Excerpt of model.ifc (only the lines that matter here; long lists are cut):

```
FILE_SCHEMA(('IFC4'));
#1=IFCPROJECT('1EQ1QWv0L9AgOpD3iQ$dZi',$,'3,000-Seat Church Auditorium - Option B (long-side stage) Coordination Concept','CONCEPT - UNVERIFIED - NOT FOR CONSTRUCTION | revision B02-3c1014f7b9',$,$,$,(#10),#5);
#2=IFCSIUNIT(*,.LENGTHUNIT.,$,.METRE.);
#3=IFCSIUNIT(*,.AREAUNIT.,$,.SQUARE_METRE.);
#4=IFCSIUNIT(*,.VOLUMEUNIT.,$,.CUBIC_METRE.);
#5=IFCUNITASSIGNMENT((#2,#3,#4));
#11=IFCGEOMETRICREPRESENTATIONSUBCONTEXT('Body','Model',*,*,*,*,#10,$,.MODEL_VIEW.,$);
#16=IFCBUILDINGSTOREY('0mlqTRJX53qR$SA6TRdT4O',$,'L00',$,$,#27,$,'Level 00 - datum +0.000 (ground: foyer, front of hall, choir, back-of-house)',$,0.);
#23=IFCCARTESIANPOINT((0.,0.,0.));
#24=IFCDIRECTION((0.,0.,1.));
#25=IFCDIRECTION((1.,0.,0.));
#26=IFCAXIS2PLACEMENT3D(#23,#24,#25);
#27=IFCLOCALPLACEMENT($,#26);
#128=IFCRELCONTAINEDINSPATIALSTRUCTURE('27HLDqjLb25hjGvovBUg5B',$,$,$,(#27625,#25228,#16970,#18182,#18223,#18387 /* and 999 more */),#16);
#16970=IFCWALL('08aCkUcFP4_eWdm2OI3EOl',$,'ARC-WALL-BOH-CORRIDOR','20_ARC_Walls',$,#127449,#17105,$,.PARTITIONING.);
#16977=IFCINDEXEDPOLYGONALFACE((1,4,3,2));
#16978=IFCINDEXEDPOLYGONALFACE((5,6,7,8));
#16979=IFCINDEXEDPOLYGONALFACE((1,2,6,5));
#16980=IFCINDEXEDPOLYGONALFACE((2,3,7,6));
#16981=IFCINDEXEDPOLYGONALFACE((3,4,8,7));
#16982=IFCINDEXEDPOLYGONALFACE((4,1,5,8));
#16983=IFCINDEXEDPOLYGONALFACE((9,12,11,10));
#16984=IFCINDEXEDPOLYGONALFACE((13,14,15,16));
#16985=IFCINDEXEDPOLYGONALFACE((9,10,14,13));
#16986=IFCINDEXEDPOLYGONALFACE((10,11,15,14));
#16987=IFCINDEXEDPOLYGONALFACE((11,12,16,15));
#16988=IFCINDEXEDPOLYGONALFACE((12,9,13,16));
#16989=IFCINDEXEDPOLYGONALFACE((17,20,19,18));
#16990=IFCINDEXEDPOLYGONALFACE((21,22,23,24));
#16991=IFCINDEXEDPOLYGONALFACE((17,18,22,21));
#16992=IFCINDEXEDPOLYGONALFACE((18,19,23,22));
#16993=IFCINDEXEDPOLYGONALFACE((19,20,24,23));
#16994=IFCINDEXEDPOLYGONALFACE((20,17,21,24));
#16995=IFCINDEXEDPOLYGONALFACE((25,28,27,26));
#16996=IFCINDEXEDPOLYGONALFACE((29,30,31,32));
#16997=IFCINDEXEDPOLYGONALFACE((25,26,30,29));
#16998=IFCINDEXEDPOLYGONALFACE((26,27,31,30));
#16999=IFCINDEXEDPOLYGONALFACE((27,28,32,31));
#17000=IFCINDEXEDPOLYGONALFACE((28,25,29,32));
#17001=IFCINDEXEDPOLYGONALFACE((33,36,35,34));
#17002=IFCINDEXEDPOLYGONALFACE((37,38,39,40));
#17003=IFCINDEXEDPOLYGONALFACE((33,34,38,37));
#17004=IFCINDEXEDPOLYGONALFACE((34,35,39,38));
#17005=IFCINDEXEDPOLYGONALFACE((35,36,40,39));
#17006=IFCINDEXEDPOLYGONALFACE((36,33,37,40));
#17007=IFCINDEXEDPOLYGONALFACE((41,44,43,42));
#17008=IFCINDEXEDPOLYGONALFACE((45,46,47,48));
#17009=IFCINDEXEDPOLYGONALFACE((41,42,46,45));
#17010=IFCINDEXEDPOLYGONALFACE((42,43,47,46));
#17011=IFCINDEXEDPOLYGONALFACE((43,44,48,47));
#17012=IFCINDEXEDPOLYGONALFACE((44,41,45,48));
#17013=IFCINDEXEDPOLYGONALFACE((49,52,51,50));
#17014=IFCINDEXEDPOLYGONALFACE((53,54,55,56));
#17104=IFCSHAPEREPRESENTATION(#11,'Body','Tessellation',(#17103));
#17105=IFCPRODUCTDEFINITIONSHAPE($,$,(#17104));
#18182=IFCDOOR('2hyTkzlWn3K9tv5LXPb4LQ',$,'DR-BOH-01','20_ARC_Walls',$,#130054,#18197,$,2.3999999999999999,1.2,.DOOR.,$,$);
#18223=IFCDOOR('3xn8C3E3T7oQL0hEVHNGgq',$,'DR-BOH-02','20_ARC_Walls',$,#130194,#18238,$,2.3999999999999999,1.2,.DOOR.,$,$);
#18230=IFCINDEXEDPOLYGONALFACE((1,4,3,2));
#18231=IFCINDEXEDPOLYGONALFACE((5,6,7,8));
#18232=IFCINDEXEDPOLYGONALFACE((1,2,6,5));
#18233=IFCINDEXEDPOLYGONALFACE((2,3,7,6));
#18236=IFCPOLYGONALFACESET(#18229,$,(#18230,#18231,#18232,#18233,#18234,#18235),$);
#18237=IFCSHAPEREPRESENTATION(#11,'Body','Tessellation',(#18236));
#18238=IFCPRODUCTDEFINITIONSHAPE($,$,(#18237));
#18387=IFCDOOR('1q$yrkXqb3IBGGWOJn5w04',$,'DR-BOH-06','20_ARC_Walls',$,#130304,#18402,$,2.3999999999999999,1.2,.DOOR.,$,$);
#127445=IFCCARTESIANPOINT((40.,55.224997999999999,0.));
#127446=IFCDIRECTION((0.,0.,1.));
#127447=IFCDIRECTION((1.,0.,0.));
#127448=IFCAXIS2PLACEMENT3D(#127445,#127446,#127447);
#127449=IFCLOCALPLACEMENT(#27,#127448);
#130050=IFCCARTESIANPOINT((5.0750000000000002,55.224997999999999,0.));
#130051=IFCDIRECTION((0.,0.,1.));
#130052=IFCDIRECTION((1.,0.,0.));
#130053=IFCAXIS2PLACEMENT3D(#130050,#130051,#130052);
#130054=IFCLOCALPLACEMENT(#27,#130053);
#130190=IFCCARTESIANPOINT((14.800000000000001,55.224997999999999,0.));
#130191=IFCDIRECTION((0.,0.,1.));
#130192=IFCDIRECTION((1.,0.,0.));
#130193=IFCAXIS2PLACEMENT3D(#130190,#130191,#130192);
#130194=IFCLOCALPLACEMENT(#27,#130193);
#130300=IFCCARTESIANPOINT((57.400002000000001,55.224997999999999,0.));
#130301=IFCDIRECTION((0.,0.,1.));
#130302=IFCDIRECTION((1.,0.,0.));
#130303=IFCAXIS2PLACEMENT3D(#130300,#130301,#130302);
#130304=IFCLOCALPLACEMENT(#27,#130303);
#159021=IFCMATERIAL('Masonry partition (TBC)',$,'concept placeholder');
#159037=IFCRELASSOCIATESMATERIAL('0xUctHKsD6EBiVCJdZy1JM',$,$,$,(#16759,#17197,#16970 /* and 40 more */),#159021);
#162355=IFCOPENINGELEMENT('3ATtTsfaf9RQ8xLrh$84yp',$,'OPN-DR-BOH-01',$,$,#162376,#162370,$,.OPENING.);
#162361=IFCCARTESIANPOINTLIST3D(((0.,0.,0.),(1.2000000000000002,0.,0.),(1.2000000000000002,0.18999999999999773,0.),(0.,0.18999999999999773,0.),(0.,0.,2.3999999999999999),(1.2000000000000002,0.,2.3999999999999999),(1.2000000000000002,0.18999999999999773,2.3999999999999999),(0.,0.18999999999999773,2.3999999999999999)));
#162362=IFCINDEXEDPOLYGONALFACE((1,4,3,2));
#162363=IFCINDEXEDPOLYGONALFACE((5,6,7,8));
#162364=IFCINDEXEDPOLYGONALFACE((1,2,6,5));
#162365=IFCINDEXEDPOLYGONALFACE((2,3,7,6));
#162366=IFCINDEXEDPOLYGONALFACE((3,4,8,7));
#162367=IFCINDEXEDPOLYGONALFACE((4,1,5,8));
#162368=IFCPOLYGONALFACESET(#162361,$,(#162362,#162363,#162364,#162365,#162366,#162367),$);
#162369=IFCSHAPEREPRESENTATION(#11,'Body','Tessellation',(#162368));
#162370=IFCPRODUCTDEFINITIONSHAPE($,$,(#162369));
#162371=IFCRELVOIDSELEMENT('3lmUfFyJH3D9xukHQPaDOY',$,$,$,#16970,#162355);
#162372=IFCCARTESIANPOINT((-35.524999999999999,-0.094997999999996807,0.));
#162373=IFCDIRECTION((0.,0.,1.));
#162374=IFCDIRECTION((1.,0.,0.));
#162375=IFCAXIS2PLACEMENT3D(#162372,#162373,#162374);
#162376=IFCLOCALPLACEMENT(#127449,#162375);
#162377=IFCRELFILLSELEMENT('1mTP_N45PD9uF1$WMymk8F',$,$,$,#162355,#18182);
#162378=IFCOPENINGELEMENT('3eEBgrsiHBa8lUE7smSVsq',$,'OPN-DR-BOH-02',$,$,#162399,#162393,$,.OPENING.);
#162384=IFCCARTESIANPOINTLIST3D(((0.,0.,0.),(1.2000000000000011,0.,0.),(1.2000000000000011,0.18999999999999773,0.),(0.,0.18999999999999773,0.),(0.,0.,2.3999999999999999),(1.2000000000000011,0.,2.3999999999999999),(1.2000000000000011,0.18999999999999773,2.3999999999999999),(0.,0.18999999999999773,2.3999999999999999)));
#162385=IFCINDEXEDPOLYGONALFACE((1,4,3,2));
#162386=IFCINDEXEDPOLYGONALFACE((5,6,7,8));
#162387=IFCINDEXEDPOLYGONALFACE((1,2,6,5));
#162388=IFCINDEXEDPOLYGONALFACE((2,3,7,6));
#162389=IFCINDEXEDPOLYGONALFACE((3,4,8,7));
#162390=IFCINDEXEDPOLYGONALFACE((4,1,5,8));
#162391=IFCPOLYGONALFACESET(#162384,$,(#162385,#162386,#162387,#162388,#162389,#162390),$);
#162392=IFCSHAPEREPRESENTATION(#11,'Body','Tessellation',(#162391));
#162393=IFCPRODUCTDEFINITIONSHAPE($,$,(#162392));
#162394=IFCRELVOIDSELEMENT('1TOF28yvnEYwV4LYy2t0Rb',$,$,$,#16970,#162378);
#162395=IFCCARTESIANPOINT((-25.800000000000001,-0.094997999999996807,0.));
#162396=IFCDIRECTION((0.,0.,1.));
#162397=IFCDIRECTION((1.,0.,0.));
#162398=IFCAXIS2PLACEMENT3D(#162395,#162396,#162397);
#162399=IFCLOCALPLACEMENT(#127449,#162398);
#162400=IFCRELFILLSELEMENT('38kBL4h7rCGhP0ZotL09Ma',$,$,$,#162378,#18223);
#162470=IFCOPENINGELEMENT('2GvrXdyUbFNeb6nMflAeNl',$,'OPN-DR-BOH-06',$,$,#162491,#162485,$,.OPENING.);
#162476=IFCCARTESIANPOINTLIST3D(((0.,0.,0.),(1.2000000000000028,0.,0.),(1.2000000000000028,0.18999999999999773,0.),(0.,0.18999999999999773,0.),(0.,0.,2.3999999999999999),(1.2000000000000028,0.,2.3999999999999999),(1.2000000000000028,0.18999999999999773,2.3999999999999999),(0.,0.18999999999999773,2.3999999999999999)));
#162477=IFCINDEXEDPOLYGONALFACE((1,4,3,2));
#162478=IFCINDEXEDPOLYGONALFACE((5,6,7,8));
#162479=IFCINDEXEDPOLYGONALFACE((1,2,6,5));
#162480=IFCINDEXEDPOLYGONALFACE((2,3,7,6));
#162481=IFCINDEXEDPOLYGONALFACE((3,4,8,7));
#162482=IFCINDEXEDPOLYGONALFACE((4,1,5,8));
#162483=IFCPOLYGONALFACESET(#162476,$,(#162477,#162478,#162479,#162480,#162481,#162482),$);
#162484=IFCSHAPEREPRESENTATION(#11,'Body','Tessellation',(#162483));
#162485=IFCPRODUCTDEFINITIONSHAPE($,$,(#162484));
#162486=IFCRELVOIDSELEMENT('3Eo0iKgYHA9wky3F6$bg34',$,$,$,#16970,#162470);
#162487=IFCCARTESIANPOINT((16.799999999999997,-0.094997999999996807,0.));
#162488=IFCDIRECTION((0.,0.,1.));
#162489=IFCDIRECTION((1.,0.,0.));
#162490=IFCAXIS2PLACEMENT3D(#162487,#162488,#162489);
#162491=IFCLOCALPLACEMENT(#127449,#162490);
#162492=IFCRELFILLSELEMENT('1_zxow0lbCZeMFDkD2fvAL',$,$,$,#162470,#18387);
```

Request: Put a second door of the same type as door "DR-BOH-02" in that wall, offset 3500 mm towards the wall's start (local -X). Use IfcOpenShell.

```python
import ifcopenshell
import ifcopenshell.api.feature
import ifcopenshell.api.geometry
import ifcopenshell.api.root
import ifcopenshell.geom
import ifcopenshell.util.element
import ifcopenshell.util.placement
import ifcopenshell.util.shape
import ifcopenshell.util.unit

model = ifcopenshell.open("model.ifc")
unit_scale = ifcopenshell.util.unit.calculate_unit_scale(model)
settings = ifcopenshell.geom.settings()


def volume(element):
    """Net volume in cubic metres, openings subtracted."""
    shape = ifcopenshell.geom.create_shape(settings, element)
    return ifcopenshell.util.shape.get_volume(shape.geometry)


door = model.by_guid("3xn8C3E3T7oQL0hEVHNGgq")
opening = door.FillsVoids[0].RelatingOpeningElement
wall = opening.VoidsElements[0].RelatingBuildingElement
before = volume(wall)
shift = ifcopenshell.util.placement.get_local_placement(wall.ObjectPlacement)[:3, 0] * -3.5 / unit_scale

# copy_class copies the void relationship, type, container and properties, but no geometry.
new_opening = ifcopenshell.api.root.copy_class(model, product=opening)
new_opening.Representation = ifcopenshell.util.element.copy_deep(
    model, opening.Representation, exclude=["IfcGeometricRepresentationContext", "IfcRepresentationMap"]
)
new_door = ifcopenshell.api.root.copy_class(model, product=door)
new_door.Representation = ifcopenshell.util.element.copy_deep(
    model, door.Representation, exclude=["IfcGeometricRepresentationContext", "IfcRepresentationMap"]
)
ifcopenshell.api.feature.add_filling(model, opening=new_opening, element=new_door)

for old, new in ((opening, new_opening), (door, new_door)):
    matrix = ifcopenshell.util.placement.get_local_placement(old.ObjectPlacement)
    matrix[:3, 3] += shift
    ifcopenshell.api.geometry.edit_object_placement(model, product=new, matrix=matrix, is_si=False)

after = volume(wall)

print(f"wall volume {before:.3f} -> {after:.3f} m3")

model.write("model_edited.ifc")
```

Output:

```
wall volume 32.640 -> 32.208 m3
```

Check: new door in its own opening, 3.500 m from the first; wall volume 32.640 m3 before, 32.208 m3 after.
